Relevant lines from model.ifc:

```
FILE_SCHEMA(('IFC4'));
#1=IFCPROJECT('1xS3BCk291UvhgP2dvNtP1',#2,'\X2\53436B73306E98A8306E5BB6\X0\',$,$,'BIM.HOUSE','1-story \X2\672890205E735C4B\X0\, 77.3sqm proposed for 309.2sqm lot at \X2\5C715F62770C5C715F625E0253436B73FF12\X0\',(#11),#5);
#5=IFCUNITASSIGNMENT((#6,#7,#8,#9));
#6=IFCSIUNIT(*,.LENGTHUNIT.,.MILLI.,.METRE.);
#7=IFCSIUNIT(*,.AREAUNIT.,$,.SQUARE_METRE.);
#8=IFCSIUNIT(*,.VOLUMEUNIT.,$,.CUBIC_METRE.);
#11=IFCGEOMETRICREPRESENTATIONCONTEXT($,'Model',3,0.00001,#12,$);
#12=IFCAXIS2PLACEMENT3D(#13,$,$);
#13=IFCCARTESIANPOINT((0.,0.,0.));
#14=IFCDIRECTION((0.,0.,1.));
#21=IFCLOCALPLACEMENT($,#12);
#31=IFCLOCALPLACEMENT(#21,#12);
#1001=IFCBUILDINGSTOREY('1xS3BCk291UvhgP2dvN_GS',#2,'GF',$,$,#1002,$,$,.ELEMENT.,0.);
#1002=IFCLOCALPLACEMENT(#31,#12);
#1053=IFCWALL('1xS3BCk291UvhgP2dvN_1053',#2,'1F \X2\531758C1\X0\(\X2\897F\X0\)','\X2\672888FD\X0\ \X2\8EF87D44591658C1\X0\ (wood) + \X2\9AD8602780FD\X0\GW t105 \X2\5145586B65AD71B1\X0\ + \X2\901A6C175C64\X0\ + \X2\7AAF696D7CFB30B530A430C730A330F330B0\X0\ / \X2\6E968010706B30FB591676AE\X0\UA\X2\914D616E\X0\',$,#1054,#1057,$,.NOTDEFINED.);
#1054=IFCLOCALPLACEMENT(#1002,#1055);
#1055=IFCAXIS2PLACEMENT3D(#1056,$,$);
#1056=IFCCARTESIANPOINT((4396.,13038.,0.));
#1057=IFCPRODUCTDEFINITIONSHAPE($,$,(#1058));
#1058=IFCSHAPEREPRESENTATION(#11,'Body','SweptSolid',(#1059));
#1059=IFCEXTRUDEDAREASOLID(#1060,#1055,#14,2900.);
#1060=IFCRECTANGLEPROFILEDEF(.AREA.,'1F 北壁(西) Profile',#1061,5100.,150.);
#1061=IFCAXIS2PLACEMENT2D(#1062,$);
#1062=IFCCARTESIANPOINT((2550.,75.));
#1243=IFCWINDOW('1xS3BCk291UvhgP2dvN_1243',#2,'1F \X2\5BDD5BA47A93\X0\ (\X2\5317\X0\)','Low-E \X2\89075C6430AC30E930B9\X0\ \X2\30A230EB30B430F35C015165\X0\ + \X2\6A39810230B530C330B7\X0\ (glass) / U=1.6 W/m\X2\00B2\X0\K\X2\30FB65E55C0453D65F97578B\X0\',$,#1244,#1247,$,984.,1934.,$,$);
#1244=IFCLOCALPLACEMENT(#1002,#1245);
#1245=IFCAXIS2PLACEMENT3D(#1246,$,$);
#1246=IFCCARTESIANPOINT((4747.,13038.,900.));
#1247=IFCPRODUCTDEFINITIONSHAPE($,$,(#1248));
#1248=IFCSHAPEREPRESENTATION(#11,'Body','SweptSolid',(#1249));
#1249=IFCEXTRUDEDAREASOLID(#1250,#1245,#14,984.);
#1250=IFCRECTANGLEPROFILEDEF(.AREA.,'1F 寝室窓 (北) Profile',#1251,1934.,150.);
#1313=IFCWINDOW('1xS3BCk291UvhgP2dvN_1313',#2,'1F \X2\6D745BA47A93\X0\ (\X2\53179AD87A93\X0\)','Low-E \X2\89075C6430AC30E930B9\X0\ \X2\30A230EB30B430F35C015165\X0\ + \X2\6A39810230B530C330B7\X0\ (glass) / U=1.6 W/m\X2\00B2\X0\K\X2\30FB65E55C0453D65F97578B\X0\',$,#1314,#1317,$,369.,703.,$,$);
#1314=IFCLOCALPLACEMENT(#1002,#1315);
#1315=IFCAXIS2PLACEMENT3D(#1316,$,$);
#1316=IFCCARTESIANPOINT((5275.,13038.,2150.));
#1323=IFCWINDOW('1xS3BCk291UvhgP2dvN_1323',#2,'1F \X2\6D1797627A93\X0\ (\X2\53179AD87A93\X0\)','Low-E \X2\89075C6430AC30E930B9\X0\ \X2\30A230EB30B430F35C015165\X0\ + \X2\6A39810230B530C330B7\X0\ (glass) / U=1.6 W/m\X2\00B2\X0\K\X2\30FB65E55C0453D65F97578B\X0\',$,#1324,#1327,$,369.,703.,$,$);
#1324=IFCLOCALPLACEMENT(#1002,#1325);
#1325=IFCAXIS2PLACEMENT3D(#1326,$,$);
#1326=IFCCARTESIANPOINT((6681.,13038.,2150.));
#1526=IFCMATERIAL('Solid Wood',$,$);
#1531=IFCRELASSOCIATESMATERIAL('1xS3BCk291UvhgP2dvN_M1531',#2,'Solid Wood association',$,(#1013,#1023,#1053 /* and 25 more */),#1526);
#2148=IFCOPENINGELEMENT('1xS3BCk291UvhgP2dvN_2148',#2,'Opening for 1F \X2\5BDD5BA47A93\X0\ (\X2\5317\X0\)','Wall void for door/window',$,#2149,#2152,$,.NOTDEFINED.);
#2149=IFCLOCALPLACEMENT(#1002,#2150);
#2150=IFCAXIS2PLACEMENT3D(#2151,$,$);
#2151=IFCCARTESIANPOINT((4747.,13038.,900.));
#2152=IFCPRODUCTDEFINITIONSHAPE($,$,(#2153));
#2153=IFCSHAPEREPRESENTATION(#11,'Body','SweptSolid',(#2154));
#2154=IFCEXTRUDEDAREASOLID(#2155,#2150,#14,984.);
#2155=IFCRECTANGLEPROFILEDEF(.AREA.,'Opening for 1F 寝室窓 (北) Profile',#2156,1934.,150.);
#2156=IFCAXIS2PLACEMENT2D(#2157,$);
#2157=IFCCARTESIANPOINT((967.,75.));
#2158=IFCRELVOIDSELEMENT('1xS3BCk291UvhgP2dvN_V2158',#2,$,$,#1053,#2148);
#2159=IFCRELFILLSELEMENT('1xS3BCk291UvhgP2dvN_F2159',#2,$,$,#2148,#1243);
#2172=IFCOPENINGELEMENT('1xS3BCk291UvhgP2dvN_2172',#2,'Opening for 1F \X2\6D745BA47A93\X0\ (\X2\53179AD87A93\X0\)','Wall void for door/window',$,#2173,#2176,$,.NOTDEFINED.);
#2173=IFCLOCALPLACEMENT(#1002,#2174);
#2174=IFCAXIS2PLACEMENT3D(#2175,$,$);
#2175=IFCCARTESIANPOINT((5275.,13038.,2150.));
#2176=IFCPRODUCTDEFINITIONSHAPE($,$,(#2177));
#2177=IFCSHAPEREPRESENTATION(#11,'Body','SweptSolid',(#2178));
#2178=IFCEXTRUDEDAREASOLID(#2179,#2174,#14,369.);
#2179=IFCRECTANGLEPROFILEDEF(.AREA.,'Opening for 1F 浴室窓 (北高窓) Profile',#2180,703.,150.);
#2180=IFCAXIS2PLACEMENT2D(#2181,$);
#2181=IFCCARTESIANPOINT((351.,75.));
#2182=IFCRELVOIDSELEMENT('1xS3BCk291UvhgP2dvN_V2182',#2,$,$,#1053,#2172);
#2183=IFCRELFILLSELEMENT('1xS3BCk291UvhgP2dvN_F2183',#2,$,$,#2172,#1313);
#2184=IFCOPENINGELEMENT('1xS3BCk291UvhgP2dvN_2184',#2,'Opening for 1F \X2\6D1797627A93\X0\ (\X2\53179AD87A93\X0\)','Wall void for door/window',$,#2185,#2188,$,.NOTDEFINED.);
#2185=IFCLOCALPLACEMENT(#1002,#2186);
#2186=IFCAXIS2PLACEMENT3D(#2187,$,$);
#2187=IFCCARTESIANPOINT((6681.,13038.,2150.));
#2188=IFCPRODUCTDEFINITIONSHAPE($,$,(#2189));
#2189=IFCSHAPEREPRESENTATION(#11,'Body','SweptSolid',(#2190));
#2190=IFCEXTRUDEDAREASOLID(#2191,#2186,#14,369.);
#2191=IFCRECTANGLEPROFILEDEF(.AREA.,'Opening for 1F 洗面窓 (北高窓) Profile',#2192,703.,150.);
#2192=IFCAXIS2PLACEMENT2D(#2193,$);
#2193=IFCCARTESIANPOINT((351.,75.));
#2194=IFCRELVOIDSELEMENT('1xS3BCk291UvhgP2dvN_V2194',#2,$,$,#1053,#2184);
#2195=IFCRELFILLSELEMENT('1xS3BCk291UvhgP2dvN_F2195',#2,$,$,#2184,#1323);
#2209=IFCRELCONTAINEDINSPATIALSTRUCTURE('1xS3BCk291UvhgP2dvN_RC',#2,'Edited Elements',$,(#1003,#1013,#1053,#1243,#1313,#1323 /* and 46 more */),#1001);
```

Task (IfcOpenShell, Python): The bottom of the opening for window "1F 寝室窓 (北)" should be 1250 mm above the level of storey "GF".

```python
import numpy as np
import ifcopenshell
import ifcopenshell.api.geometry
import ifcopenshell.geom
import ifcopenshell.util.element
import ifcopenshell.util.placement
import ifcopenshell.util.shape
import ifcopenshell.util.unit

model = ifcopenshell.open("model.ifc")
unit_scale = ifcopenshell.util.unit.calculate_unit_scale(model)

window = model.by_id(1243)
opening = window.FillsVoids[0].RelatingOpeningElement
storey = ifcopenshell.util.element.get_container(window, ifc_class="IfcBuildingStorey")
level = ifcopenshell.util.placement.get_local_placement(storey.ObjectPlacement)[2, 3]

# The opening's origin need not be at the sill, so measure its lowest point.
shape = ifcopenshell.geom.create_shape(ifcopenshell.geom.settings(), opening)
bottom = ifcopenshell.util.shape.get_shape_bottom_elevation(shape, shape.geometry) / unit_scale
dz = level + 1.25 / unit_scale - bottom

shift = np.array([0.0, 0.0, dz])
# The window is not placed relative to its opening, so move both.
for product in (opening, window):
    matrix = ifcopenshell.util.placement.get_local_placement(product.ObjectPlacement)
    matrix[:3, 3] += shift
    ifcopenshell.api.geometry.edit_object_placement(model, product=product, matrix=matrix, is_si=False)

print(f"moved by {dz * unit_scale:+.3f} m")

model.write("model_rev.ifc")
```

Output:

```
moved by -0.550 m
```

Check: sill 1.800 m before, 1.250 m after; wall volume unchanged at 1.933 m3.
